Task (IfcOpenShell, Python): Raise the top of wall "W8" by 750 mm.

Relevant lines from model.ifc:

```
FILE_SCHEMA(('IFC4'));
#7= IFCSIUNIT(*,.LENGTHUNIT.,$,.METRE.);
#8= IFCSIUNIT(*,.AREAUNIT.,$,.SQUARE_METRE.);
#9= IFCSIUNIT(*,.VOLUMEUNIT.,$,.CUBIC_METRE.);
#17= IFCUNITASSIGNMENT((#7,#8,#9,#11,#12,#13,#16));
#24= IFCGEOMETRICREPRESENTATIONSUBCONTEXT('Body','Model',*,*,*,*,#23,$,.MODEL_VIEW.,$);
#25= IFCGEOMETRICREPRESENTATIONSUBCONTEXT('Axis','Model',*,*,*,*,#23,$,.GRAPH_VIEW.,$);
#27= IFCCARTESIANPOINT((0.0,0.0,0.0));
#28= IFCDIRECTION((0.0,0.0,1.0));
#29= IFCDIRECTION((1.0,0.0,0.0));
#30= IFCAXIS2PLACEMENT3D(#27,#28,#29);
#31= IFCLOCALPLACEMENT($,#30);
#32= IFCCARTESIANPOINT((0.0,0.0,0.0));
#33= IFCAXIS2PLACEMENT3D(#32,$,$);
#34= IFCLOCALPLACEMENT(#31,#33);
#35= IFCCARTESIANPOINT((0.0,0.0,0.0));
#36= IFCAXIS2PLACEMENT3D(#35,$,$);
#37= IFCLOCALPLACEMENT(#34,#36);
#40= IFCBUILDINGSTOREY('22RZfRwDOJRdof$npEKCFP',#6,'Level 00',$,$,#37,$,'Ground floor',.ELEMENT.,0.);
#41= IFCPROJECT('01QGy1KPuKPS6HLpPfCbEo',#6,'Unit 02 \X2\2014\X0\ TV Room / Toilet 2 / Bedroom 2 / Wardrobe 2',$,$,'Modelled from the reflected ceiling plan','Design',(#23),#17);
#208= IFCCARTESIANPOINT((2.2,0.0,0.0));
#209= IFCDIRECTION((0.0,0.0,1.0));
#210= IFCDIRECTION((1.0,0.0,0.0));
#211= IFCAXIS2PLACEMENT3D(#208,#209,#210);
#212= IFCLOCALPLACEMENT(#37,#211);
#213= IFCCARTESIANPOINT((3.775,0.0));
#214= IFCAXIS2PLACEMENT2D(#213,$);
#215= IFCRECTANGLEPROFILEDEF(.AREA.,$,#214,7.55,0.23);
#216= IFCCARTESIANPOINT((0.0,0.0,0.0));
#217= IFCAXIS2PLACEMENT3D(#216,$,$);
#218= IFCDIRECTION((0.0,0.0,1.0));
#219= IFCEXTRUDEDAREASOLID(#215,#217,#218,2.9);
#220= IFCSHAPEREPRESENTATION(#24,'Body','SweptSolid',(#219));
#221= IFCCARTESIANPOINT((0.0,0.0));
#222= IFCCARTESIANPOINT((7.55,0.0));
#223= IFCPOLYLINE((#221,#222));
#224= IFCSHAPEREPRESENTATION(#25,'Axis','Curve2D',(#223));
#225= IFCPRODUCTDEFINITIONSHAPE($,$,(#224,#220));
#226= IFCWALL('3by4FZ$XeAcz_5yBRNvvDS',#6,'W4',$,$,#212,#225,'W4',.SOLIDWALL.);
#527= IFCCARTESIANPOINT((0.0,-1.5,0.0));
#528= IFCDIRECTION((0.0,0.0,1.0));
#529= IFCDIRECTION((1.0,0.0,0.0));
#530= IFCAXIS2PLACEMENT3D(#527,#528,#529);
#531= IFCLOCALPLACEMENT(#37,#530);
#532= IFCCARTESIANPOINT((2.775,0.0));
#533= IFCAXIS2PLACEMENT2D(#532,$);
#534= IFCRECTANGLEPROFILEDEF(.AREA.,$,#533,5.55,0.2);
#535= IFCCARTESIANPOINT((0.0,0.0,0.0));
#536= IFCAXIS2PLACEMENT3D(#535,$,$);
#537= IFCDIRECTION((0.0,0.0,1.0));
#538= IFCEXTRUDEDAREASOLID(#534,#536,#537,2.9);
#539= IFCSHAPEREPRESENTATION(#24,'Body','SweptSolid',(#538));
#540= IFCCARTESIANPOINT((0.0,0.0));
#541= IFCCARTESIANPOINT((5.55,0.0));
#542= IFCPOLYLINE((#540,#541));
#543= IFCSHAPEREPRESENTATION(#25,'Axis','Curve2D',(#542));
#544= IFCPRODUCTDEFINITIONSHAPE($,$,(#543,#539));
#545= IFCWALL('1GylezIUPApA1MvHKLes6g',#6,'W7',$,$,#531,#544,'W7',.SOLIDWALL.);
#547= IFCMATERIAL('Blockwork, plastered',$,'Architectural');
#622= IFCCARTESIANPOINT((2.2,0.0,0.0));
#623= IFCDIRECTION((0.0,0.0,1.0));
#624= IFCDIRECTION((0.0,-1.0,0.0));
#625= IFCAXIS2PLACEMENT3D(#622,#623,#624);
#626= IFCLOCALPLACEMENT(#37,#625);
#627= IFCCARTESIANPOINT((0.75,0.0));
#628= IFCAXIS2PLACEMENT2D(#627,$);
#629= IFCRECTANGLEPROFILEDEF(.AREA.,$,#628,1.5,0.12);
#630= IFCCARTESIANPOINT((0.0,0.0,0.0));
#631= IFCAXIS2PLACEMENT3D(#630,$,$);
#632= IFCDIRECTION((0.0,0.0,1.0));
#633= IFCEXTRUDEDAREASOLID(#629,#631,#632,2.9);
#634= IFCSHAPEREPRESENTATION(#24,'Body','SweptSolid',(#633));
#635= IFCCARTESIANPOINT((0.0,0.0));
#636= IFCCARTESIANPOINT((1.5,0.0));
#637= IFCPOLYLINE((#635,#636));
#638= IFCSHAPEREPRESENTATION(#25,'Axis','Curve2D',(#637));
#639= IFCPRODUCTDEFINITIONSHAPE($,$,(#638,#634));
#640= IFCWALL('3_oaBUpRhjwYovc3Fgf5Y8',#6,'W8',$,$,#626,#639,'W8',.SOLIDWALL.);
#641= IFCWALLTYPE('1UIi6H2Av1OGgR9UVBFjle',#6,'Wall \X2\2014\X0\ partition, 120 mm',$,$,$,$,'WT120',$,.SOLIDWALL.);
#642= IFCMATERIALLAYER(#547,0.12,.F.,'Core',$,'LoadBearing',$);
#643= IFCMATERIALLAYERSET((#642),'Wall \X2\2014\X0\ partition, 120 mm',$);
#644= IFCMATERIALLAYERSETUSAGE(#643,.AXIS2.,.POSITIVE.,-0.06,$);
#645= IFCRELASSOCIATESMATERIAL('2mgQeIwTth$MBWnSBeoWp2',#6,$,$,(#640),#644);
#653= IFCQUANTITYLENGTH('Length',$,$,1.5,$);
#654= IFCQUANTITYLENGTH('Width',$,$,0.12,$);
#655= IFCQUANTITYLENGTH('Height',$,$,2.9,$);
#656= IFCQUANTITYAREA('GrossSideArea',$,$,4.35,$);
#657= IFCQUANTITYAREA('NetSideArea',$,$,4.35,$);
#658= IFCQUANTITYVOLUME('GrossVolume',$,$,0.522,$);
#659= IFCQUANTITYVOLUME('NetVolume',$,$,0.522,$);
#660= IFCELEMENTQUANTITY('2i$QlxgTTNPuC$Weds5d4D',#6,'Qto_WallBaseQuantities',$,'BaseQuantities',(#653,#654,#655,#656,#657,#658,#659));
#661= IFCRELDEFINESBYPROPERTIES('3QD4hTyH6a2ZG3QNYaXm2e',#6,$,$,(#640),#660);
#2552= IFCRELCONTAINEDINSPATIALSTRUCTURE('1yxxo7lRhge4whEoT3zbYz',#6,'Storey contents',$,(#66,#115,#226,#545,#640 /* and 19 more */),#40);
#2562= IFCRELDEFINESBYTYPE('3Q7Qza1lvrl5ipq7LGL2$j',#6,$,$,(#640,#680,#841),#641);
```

```python
import ifcopenshell
import ifcopenshell.api.pset
import ifcopenshell.geom
import ifcopenshell.util.element
import ifcopenshell.util.representation
import ifcopenshell.util.shape
import ifcopenshell.util.unit

model = ifcopenshell.open("model.ifc")
unit_scale = ifcopenshell.util.unit.calculate_unit_scale(model)
area_scale = ifcopenshell.util.unit.calculate_unit_scale(model, "AREAUNIT")
volume_scale = ifcopenshell.util.unit.calculate_unit_scale(model, "VOLUMEUNIT")
settings = ifcopenshell.geom.settings()


def volume(element):
    """Net volume in cubic metres, openings subtracted."""
    shape = ifcopenshell.geom.create_shape(settings, element)
    return ifcopenshell.util.shape.get_volume(shape.geometry)


wall = model.by_id(640)
before = volume(wall)

body = ifcopenshell.util.representation.get_representation(wall, "Model", "Body")
solid = body.Items[0]
old_height = solid.Depth
solid.Depth += 0.75
after = volume(wall)
thickness = 0.12  # wall thickness in metres

# Update the stored height, areas and volumes.
qto = model.by_id(ifcopenshell.util.element.get_pset(wall, "Qto_WallBaseQuantities", should_inherit=False)["id"])
ifcopenshell.api.pset.edit_qto(model, qto=qto, properties={
    "Height": solid.Depth,
    "GrossSideArea": ifcopenshell.util.element.get_pset(wall, "Qto_WallBaseQuantities", "GrossSideArea") * solid.Depth / old_height,
    "NetSideArea": after / thickness / area_scale,
    "GrossVolume": ifcopenshell.util.element.get_pset(wall, "Qto_WallBaseQuantities", "GrossVolume") * solid.Depth / old_height,
    "NetVolume": after / volume_scale,
})

print(f"height {old_height:g} -> {solid.Depth:g}, volume {before:.3f} -> {after:.3f} m3")

model.write("model_edited.ifc")
```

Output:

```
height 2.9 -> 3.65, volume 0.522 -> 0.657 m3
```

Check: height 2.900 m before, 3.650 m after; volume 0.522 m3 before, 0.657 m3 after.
